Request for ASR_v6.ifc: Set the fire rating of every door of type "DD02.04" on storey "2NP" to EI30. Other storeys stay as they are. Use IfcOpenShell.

First a look at what the model holds.

```python
import ifcopenshell
import ifcopenshell.util.element

model = ifcopenshell.open("ASR_v6.ifc")
print(model.schema)
storey = next(s for s in model.by_type("IfcBuildingStorey") if s.Name == "2NP")
doors = [e for e in ifcopenshell.util.element.get_decomposition(storey) if e.is_a("IfcDoor")]
seen = {}
for e in doors:
    element_type = ifcopenshell.util.element.get_type(e)
    key = (element_type.Name if element_type != e and element_type else None, ifcopenshell.util.element.get_pset(e, "Pset_DoorCommon", "FireRating"))
    seen[key] = seen.get(key, 0) + 1
for (name, value), count in sorted(seen.items(), key=str):
    print(count, "x", name, "|", value)
```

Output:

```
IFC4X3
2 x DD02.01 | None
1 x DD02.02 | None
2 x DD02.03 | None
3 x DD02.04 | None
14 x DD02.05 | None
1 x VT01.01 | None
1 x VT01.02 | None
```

```python
import ifcopenshell
import ifcopenshell.api.pset
import ifcopenshell.util.element

model = ifcopenshell.open("ASR_v6.ifc")

storey = next(s for s in model.by_type("IfcBuildingStorey") if s.Name == "2NP")
doors = [e for e in ifcopenshell.util.element.get_decomposition(storey) if e.is_a("IfcDoor")]

count = 0
for e in doors:
    element_type = ifcopenshell.util.element.get_type(e)
    if element_type in (None, e) or element_type.Name != "DD02.04":
        continue
    # add_pset returns the element's existing set when there is one.
    pset = ifcopenshell.api.pset.add_pset(model, product=e, name="Pset_DoorCommon")
    ifcopenshell.api.pset.edit_pset(model, pset=pset, properties={"FireRating": "EI30"})
    count += 1

print(count, "doors updated")

model.write("ASR_v6_edited.ifc")
```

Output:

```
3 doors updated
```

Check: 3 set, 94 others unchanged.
